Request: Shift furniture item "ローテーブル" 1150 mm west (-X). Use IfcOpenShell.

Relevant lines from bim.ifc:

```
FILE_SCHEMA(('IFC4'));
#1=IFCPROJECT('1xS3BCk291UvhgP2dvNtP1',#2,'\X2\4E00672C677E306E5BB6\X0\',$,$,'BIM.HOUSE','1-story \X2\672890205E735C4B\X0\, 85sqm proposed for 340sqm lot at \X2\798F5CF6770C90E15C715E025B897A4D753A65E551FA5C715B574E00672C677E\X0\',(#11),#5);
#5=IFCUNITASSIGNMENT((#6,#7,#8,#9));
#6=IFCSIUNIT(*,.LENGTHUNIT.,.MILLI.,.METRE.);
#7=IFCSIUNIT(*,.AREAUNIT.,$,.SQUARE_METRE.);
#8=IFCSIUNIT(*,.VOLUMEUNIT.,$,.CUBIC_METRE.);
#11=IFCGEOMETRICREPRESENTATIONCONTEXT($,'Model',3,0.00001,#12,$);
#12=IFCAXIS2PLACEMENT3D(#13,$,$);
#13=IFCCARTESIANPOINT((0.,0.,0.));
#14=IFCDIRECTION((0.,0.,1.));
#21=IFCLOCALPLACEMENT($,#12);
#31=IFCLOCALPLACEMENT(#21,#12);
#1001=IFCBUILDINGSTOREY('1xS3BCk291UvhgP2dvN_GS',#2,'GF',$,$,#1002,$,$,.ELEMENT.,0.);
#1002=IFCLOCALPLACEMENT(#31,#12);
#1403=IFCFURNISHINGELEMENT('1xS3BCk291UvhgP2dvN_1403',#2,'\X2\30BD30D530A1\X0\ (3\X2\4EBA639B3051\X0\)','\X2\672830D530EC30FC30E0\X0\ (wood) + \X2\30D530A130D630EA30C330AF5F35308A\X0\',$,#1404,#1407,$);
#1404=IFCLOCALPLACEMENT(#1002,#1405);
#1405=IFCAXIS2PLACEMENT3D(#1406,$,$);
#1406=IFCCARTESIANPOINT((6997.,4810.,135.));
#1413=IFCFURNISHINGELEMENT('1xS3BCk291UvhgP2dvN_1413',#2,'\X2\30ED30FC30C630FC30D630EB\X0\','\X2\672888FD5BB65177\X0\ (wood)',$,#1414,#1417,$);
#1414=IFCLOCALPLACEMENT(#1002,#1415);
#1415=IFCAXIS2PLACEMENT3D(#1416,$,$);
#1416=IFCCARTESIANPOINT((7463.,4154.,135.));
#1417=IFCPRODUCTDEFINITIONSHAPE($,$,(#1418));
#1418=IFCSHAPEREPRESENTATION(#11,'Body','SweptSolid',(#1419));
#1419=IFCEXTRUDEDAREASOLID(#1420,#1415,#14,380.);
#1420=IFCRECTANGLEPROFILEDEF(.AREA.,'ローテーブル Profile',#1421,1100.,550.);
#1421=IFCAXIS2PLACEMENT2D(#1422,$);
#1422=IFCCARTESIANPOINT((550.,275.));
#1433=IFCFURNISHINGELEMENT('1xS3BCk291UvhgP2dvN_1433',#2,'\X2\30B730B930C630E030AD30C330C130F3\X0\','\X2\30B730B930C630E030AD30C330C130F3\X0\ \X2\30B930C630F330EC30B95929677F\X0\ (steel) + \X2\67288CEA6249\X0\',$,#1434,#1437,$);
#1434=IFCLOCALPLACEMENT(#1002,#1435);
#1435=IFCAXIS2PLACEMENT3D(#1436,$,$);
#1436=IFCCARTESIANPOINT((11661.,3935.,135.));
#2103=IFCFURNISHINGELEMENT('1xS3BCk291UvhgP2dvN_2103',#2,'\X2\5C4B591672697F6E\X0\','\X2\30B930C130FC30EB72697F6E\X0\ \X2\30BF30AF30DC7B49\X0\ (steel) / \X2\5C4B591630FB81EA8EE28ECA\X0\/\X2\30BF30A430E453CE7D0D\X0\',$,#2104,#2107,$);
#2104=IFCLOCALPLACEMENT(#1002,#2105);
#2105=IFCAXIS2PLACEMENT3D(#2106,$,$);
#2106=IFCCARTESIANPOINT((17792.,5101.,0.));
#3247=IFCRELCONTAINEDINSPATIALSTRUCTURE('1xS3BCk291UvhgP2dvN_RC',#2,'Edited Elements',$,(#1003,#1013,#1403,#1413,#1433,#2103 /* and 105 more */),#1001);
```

```python
import ifcopenshell
import ifcopenshell.api.geometry
import ifcopenshell.util.placement
import ifcopenshell.util.unit

model = ifcopenshell.open("bim.ifc")
unit_scale = ifcopenshell.util.unit.calculate_unit_scale(model)

item = model.by_guid("1xS3BCk291UvhgP2dvN_1413")
matrix = ifcopenshell.util.placement.get_local_placement(item.ObjectPlacement)
matrix[0, 3] -= 1.15 / unit_scale
ifcopenshell.api.geometry.edit_object_placement(model, product=item, matrix=matrix, is_si=False)

print(ifcopenshell.util.placement.get_local_placement(item.ObjectPlacement).round(3) + 0.0)

model.write("bim_edited.ifc")
```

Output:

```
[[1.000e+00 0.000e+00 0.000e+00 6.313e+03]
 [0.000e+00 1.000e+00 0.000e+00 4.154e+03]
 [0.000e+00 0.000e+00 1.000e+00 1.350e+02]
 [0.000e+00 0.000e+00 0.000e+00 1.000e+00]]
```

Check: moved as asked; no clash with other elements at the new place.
